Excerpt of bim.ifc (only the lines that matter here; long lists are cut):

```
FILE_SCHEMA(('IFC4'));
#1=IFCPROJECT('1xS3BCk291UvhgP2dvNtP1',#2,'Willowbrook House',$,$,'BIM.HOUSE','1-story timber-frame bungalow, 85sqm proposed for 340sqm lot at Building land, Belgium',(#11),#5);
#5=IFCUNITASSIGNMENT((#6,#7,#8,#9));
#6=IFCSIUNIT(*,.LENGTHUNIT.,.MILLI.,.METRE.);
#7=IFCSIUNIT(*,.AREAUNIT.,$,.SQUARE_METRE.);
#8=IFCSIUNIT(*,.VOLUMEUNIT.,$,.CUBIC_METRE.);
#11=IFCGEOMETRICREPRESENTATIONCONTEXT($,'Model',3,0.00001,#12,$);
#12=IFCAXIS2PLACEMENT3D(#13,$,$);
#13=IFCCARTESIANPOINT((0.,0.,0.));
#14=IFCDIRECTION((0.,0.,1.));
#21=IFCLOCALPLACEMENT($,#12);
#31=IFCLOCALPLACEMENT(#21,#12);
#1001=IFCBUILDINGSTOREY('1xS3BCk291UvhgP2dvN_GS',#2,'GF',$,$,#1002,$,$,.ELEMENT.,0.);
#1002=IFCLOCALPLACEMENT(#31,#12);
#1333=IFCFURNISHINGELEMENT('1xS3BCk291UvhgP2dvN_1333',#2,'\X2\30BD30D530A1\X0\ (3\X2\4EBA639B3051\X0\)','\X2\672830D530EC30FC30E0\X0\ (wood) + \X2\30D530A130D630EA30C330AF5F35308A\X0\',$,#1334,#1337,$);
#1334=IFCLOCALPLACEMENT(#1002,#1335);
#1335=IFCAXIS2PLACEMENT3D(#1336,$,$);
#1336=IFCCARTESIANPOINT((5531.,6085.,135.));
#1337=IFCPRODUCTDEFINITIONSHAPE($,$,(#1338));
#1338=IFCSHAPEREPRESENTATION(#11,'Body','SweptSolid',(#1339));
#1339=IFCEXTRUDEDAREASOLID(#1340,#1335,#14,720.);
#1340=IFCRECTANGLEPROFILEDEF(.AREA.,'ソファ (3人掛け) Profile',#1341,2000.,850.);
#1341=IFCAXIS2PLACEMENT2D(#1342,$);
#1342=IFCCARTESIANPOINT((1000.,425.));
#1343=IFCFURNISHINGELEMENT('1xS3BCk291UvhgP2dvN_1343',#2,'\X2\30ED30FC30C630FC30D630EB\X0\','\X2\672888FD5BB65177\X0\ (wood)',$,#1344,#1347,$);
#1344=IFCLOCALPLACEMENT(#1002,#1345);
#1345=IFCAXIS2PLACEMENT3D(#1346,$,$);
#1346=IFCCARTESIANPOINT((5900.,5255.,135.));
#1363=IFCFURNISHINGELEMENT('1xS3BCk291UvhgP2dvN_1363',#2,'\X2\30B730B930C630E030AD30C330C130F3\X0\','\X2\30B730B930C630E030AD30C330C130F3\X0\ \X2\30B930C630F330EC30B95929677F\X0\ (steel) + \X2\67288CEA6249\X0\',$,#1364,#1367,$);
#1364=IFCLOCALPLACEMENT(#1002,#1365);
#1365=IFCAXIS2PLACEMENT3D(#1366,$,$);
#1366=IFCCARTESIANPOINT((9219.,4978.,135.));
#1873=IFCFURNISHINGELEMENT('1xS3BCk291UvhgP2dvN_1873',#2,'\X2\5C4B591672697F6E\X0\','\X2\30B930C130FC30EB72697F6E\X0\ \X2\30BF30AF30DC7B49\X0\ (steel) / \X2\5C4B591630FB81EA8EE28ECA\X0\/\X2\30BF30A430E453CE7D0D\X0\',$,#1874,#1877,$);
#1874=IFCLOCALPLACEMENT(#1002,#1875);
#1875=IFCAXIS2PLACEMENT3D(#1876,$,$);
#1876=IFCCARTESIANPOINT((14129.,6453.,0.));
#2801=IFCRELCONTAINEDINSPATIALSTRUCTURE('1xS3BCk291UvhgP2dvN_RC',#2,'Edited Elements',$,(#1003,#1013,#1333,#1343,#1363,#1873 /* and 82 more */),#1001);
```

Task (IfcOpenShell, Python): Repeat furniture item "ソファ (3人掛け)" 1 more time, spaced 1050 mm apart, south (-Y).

```python
import numpy as np
import ifcopenshell
import ifcopenshell.api.geometry
import ifcopenshell.api.root
import ifcopenshell.util.element
import ifcopenshell.util.placement
import ifcopenshell.util.unit

model = ifcopenshell.open("bim.ifc")
unit_scale = ifcopenshell.util.unit.calculate_unit_scale(model)


def reuse_history(source, copy):
    """copy_class also copies each property set's owner history, people and application; keep the originals."""
    for rel in copy.IsDefinedBy:
        if rel.is_a("IfcRelDefinesByProperties") and (history := rel.RelatingPropertyDefinition.OwnerHistory):
            rel.RelatingPropertyDefinition.OwnerHistory = source.OwnerHistory
            ifcopenshell.util.element.remove_deep2(model, history)


source = model.by_guid("1xS3BCk291UvhgP2dvN_1333")
base = ifcopenshell.util.placement.get_local_placement(source.ObjectPlacement)
step = np.array([0.0, -1.0, 0.0]) * 1.05 / unit_scale

for i in range(1, 2):
    copy = ifcopenshell.api.root.copy_class(model, product=source)
    copy.Representation = ifcopenshell.util.element.copy_deep(
        model, source.Representation, exclude=["IfcGeometricRepresentationContext", "IfcRepresentationMap"]
    )
    reuse_history(source, copy)
    matrix = base.copy()
    matrix[:3, 3] += i * step
    print("added at", matrix[:3, 3].round(3) + 0.0)
    ifcopenshell.api.geometry.edit_object_placement(model, product=copy, matrix=matrix, is_si=False)

model.write("bim-out.ifc")
```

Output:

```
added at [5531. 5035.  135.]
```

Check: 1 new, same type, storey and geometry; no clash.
